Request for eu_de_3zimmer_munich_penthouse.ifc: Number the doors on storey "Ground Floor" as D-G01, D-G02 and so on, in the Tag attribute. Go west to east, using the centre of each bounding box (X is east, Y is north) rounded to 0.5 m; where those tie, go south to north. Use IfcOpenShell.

First a look at what the model holds.

```python
import ifcopenshell
import ifcopenshell.util.element
import ifcopenshell.util.placement

model = ifcopenshell.open("eu_de_3zimmer_munich_penthouse.ifc")
print(model.schema)
storey = next(s for s in model.by_type("IfcBuildingStorey") if s.Name == "Ground Floor")
doors = [e for e in ifcopenshell.util.element.get_decomposition(storey) if e.is_a("IfcDoor")]
for e in sorted(doors, key=lambda e: e.id()):
    origin = ifcopenshell.util.placement.get_local_placement(e.ObjectPlacement)[:3, 3]
    print(e.id(), e.Tag, e.Name, origin.round(2) + 0.0, sep=" | ")
```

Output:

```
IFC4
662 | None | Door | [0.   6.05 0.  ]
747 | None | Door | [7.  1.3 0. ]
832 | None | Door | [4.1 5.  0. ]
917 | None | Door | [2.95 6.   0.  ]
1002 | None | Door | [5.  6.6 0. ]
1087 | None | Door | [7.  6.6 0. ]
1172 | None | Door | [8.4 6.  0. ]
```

```python
import ifcopenshell
import ifcopenshell.geom
import ifcopenshell.util.element
import ifcopenshell.util.shape

model = ifcopenshell.open("eu_de_3zimmer_munich_penthouse.ifc")
settings = ifcopenshell.geom.settings()
settings.set("use-world-coords", True)


def centre(element):
    shape = ifcopenshell.geom.create_shape(settings, element)
    return ifcopenshell.util.shape.get_bbox_centroid(shape.geometry)


storey = next(s for s in model.by_type("IfcBuildingStorey") if s.Name == "Ground Floor")
doors = [e for e in ifcopenshell.util.element.get_decomposition(storey) if e.is_a("IfcDoor")]

# Insertion points can sit at a corner or the storey origin, so sort by the geometry (in metres).
centres = {e: centre(e) for e in doors}
doors.sort(key=lambda e: (round(centres[e][0] / 0.5), centres[e][1]))

for i, e in enumerate(doors, start=1):
    number = f"D-G{i:02d}"
    e.Tag = number
    print(e.id(), number)

model.write("eu_de_3zimmer_munich_penthouse-out.ifc")
```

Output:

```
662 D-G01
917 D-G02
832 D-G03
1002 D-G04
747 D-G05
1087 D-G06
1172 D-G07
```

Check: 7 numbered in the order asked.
